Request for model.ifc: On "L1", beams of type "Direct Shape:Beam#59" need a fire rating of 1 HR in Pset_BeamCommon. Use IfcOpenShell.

First a look at what the model holds.

```python
import ifcopenshell
import ifcopenshell.util.element

model = ifcopenshell.open("model.ifc")
print(model.schema)
storey = next(s for s in model.by_type("IfcBuildingStorey") if s.Name == "L1")
beams = [e for e in ifcopenshell.util.element.get_decomposition(storey) if e.is_a("IfcBeam")]
seen = {}
for e in beams:
    element_type = ifcopenshell.util.element.get_type(e)
    key = (element_type.Name if element_type != e and element_type else None, ifcopenshell.util.element.get_pset(e, "Pset_BeamCommon", "FireRating"))
    seen[key] = seen.get(key, 0) + 1
for (name, value), count in sorted(seen.items(), key=str):
    print(count, "x", name, "|", value)
```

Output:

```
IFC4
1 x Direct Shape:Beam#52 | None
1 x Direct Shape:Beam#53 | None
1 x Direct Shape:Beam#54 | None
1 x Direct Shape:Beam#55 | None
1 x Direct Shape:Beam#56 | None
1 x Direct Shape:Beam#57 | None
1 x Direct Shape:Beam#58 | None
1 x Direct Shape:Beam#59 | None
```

```python
import ifcopenshell
import ifcopenshell.api.pset
import ifcopenshell.util.element

model = ifcopenshell.open("model.ifc")

storey = next(s for s in model.by_type("IfcBuildingStorey") if s.Name == "L1")
beams = [e for e in ifcopenshell.util.element.get_decomposition(storey) if e.is_a("IfcBeam")]

count = 0
for e in beams:
    element_type = ifcopenshell.util.element.get_type(e)
    if element_type in (None, e) or element_type.Name != "Direct Shape:Beam#59":
        continue
    # add_pset returns the element's existing set when there is one.
    pset = ifcopenshell.api.pset.add_pset(model, product=e, name="Pset_BeamCommon")
    ifcopenshell.api.pset.edit_pset(model, pset=pset, properties={"FireRating": "1 HR"})
    count += 1

print(count, "beams updated")

model.write("model-out.ifc")
```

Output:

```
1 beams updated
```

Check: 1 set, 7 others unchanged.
